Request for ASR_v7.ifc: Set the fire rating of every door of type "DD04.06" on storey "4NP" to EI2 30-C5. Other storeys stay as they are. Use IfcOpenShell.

First a look at what the model holds.

```python
import ifcopenshell
import ifcopenshell.util.element

model = ifcopenshell.open("ASR_v7.ifc")
print(model.schema)
storey = next(s for s in model.by_type("IfcBuildingStorey") if s.Name == "4NP")
doors = [e for e in ifcopenshell.util.element.get_decomposition(storey) if e.is_a("IfcDoor")]
seen = {}
for e in doors:
    element_type = ifcopenshell.util.element.get_type(e)
    key = (element_type.Name if element_type != e and element_type else None, ifcopenshell.util.element.get_pset(e, "Pset_DoorCommon", "FireRating"))
    seen[key] = seen.get(key, 0) + 1
for (name, value), count in sorted(seen.items(), key=str):
    print(count, "x", name, "|", value)
```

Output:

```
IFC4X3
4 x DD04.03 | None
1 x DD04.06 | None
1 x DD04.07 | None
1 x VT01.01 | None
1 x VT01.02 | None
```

```python
import ifcopenshell
import ifcopenshell.api.pset
import ifcopenshell.util.element

model = ifcopenshell.open("ASR_v7.ifc")

storey = next(s for s in model.by_type("IfcBuildingStorey") if s.Name == "4NP")
doors = [e for e in ifcopenshell.util.element.get_decomposition(storey) if e.is_a("IfcDoor")]

count = 0
for e in doors:
    element_type = ifcopenshell.util.element.get_type(e)
    if element_type in (None, e) or element_type.Name != "DD04.06":
        continue
    # add_pset returns the element's existing set when there is one.
    pset = ifcopenshell.api.pset.add_pset(model, product=e, name="Pset_DoorCommon")
    ifcopenshell.api.pset.edit_pset(model, pset=pset, properties={"FireRating": "EI2 30-C5"})
    count += 1

print(count, "doors updated")

model.write("ASR_v7-out.ifc")
```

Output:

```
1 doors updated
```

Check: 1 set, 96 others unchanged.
